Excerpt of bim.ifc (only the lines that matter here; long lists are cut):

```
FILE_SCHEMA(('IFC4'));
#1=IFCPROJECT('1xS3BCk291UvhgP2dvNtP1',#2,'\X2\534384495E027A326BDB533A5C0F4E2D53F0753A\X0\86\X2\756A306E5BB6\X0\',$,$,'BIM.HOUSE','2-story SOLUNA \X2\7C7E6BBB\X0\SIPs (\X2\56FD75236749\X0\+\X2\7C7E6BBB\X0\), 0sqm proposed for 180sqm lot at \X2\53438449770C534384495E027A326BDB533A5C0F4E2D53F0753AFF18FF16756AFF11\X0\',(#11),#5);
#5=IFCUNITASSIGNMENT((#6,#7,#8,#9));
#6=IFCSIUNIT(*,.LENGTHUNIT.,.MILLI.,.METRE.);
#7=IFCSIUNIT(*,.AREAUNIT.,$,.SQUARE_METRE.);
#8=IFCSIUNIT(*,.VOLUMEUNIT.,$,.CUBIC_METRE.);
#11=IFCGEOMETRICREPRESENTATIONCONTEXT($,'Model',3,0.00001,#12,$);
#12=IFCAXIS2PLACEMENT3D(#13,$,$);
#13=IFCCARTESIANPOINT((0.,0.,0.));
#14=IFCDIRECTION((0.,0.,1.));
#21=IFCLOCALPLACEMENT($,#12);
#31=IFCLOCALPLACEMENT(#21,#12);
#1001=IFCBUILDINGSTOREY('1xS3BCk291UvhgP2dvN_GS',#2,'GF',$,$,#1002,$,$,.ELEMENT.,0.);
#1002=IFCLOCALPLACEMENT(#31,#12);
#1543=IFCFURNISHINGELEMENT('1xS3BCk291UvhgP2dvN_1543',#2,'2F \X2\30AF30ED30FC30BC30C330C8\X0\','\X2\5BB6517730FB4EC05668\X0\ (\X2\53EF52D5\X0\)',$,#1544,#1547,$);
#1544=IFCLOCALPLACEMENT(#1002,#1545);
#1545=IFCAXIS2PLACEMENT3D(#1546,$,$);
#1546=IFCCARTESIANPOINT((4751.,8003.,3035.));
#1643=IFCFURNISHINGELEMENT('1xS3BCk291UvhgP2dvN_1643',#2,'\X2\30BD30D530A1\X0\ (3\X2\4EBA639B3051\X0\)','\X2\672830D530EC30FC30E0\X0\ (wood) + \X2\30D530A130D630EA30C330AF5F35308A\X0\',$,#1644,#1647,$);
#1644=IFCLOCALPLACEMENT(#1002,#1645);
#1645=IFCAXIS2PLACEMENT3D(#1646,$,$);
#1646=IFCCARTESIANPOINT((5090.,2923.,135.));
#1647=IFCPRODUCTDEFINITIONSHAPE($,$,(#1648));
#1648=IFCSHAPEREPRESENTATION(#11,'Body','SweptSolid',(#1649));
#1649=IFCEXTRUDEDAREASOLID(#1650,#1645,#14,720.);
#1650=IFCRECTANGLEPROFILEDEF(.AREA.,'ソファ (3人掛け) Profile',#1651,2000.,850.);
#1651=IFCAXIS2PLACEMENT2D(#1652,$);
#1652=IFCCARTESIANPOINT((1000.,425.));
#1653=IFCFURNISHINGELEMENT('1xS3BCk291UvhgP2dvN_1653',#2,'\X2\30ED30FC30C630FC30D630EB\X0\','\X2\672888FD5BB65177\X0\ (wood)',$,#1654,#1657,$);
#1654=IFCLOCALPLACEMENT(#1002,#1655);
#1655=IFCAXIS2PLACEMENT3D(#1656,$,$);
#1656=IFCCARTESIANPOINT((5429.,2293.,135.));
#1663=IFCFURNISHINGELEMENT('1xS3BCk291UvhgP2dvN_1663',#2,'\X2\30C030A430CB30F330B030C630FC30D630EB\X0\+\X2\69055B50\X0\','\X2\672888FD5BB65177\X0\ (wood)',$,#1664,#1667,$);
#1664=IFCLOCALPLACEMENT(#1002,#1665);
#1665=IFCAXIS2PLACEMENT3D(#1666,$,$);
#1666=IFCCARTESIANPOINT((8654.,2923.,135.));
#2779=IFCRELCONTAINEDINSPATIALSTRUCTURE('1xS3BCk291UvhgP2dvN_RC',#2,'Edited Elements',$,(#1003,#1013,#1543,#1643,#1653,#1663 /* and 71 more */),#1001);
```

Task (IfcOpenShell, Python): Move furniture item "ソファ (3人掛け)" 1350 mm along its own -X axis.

```python
import ifcopenshell
import ifcopenshell.api.geometry
import ifcopenshell.util.placement

model = ifcopenshell.open("bim.ifc")

item = model.by_id(1643)
matrix = ifcopenshell.util.placement.get_local_placement(item.ObjectPlacement)
matrix[:3, 3] -= matrix[:3, 0] * 1350.0
ifcopenshell.api.geometry.edit_object_placement(model, product=item, matrix=matrix, is_si=False)

print(ifcopenshell.util.placement.get_local_placement(item.ObjectPlacement).round(3) + 0.0)

model.write("bim_updated.ifc")
```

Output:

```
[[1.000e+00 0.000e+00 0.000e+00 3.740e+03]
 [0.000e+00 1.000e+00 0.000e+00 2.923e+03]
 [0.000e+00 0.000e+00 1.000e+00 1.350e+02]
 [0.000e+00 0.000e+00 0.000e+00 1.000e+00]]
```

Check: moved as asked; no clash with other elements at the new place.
